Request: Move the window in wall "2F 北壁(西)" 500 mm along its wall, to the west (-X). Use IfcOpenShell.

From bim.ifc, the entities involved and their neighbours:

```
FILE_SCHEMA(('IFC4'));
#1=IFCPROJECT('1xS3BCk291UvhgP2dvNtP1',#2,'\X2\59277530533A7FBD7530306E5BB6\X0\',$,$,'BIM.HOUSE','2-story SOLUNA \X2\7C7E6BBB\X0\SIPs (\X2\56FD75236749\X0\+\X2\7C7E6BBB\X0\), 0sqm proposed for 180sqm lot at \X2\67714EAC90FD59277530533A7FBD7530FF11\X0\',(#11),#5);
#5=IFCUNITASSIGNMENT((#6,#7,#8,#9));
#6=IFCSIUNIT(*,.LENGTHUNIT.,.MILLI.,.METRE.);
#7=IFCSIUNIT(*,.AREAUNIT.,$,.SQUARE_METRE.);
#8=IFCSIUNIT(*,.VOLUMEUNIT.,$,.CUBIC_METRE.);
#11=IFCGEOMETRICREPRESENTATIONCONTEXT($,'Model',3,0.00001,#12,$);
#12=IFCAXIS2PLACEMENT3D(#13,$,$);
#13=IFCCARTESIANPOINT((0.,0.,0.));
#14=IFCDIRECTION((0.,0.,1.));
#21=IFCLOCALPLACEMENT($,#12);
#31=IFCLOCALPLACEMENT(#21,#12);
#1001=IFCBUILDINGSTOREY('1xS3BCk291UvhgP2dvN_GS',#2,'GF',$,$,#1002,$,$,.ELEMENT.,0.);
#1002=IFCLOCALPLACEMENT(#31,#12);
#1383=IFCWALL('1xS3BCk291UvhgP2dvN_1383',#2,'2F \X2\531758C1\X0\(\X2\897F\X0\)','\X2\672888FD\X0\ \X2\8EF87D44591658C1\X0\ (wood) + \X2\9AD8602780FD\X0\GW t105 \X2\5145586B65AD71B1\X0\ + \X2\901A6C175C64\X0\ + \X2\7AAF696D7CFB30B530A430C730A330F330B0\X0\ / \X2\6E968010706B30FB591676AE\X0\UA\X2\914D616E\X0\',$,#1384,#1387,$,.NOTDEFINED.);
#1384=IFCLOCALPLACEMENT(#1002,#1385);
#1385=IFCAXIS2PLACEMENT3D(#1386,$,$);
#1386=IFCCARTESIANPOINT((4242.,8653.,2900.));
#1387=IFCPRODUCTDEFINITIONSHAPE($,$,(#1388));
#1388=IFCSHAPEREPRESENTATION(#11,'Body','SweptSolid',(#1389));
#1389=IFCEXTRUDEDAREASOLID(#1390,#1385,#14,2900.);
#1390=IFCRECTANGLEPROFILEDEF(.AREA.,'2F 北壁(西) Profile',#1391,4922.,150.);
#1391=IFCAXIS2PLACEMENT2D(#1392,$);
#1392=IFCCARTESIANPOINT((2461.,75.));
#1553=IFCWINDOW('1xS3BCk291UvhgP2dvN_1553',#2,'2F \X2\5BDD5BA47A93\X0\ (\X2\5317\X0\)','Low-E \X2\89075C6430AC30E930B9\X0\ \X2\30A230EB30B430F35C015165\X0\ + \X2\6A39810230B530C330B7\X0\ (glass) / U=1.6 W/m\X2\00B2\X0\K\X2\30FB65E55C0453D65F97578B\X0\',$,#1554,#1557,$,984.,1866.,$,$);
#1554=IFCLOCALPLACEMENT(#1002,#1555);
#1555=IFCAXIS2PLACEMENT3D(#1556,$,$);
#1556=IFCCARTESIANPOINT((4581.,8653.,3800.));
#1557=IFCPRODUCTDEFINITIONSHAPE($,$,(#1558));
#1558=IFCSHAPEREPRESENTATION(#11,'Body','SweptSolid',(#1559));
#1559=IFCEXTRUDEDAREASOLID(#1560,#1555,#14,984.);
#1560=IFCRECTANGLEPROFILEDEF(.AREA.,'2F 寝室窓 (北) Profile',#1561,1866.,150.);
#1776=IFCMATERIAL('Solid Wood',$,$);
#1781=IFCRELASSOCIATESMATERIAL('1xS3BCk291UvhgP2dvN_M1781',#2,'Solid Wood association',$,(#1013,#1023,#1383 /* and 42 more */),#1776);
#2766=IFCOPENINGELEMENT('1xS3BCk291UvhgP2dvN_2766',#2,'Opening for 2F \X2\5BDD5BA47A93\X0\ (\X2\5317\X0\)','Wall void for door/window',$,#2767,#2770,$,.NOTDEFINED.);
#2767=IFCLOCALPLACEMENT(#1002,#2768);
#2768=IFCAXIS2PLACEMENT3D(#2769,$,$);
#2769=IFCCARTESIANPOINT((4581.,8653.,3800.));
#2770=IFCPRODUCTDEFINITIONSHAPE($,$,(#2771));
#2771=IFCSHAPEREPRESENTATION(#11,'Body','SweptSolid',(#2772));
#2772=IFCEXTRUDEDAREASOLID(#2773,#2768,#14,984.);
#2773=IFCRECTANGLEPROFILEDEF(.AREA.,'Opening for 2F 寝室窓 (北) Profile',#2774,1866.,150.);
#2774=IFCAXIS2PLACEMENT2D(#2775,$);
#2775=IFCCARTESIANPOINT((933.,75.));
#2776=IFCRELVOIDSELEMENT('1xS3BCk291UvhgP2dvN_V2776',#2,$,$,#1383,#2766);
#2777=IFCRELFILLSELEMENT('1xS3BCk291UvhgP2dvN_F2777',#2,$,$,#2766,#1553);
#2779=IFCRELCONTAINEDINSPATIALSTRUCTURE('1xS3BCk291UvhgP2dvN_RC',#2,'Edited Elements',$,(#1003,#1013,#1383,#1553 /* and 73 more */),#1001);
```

```python
import ifcopenshell
import ifcopenshell.api.geometry
import ifcopenshell.util.placement

model = ifcopenshell.open("bim.ifc")

window = model.by_guid("1xS3BCk291UvhgP2dvN_1553")
opening = window.FillsVoids[0].RelatingOpeningElement
wall = opening.VoidsElements[0].RelatingBuildingElement

wall_matrix = ifcopenshell.util.placement.get_local_placement(wall.ObjectPlacement)
shift = wall_matrix[:3, 0] * -500.0
before = ifcopenshell.util.placement.get_local_placement(window.ObjectPlacement)[:3, 3].copy()

# The window is not placed relative to its opening, so move both.
for product in (opening, window):
    matrix = ifcopenshell.util.placement.get_local_placement(product.ObjectPlacement)
    matrix[:3, 3] += shift
    ifcopenshell.api.geometry.edit_object_placement(model, product=product, matrix=matrix, is_si=False)

after = ifcopenshell.util.placement.get_local_placement(window.ObjectPlacement)[:3, 3]
print("window moved by", (after - before).round(3) + 0.0)

model.write("bim_edited.ifc")
```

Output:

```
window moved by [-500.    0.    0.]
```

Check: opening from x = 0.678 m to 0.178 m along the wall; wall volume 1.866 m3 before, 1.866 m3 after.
